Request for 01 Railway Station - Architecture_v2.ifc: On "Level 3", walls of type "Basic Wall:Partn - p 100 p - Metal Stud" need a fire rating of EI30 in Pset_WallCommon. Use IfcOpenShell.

First a look at what the model holds.

```python
import ifcopenshell
import ifcopenshell.util.element

model = ifcopenshell.open("01 Railway Station - Architecture_v2.ifc")
print(model.schema)
storey = next(s for s in model.by_type("IfcBuildingStorey") if s.Name == "Level 3")
walls = [e for e in ifcopenshell.util.element.get_decomposition(storey) if e.is_a("IfcWall")]
seen = {}
for e in walls:
    element_type = ifcopenshell.util.element.get_type(e)
    key = (element_type.Name if element_type != e and element_type else None, ifcopenshell.util.element.get_pset(e, "Pset_WallCommon", "FireRating"))
    seen[key] = seen.get(key, 0) + 1
for (name, value), count in sorted(seen.items(), key=str):
    print(count, "x", name, "|", value)
```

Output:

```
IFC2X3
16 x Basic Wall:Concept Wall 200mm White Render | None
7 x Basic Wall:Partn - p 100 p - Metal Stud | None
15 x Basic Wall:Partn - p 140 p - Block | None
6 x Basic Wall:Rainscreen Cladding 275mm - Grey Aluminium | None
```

```python
import ifcopenshell
import ifcopenshell.api.pset
import ifcopenshell.util.element

model = ifcopenshell.open("01 Railway Station - Architecture_v2.ifc")

storey = next(s for s in model.by_type("IfcBuildingStorey") if s.Name == "Level 3")
walls = [e for e in ifcopenshell.util.element.get_decomposition(storey) if e.is_a("IfcWall")]

count = 0
for e in walls:
    element_type = ifcopenshell.util.element.get_type(e)
    if element_type in (None, e) or element_type.Name != "Basic Wall:Partn - p 100 p - Metal Stud":
        continue
    # add_pset returns the element's existing set when there is one.
    pset = ifcopenshell.api.pset.add_pset(model, product=e, name="Pset_WallCommon")
    ifcopenshell.api.pset.edit_pset(model, pset=pset, properties={"FireRating": "EI30"})
    count += 1

print(count, "walls updated")

model.write("01 Railway Station - Architecture_v2_v2.ifc")
```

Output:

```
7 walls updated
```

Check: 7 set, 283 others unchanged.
